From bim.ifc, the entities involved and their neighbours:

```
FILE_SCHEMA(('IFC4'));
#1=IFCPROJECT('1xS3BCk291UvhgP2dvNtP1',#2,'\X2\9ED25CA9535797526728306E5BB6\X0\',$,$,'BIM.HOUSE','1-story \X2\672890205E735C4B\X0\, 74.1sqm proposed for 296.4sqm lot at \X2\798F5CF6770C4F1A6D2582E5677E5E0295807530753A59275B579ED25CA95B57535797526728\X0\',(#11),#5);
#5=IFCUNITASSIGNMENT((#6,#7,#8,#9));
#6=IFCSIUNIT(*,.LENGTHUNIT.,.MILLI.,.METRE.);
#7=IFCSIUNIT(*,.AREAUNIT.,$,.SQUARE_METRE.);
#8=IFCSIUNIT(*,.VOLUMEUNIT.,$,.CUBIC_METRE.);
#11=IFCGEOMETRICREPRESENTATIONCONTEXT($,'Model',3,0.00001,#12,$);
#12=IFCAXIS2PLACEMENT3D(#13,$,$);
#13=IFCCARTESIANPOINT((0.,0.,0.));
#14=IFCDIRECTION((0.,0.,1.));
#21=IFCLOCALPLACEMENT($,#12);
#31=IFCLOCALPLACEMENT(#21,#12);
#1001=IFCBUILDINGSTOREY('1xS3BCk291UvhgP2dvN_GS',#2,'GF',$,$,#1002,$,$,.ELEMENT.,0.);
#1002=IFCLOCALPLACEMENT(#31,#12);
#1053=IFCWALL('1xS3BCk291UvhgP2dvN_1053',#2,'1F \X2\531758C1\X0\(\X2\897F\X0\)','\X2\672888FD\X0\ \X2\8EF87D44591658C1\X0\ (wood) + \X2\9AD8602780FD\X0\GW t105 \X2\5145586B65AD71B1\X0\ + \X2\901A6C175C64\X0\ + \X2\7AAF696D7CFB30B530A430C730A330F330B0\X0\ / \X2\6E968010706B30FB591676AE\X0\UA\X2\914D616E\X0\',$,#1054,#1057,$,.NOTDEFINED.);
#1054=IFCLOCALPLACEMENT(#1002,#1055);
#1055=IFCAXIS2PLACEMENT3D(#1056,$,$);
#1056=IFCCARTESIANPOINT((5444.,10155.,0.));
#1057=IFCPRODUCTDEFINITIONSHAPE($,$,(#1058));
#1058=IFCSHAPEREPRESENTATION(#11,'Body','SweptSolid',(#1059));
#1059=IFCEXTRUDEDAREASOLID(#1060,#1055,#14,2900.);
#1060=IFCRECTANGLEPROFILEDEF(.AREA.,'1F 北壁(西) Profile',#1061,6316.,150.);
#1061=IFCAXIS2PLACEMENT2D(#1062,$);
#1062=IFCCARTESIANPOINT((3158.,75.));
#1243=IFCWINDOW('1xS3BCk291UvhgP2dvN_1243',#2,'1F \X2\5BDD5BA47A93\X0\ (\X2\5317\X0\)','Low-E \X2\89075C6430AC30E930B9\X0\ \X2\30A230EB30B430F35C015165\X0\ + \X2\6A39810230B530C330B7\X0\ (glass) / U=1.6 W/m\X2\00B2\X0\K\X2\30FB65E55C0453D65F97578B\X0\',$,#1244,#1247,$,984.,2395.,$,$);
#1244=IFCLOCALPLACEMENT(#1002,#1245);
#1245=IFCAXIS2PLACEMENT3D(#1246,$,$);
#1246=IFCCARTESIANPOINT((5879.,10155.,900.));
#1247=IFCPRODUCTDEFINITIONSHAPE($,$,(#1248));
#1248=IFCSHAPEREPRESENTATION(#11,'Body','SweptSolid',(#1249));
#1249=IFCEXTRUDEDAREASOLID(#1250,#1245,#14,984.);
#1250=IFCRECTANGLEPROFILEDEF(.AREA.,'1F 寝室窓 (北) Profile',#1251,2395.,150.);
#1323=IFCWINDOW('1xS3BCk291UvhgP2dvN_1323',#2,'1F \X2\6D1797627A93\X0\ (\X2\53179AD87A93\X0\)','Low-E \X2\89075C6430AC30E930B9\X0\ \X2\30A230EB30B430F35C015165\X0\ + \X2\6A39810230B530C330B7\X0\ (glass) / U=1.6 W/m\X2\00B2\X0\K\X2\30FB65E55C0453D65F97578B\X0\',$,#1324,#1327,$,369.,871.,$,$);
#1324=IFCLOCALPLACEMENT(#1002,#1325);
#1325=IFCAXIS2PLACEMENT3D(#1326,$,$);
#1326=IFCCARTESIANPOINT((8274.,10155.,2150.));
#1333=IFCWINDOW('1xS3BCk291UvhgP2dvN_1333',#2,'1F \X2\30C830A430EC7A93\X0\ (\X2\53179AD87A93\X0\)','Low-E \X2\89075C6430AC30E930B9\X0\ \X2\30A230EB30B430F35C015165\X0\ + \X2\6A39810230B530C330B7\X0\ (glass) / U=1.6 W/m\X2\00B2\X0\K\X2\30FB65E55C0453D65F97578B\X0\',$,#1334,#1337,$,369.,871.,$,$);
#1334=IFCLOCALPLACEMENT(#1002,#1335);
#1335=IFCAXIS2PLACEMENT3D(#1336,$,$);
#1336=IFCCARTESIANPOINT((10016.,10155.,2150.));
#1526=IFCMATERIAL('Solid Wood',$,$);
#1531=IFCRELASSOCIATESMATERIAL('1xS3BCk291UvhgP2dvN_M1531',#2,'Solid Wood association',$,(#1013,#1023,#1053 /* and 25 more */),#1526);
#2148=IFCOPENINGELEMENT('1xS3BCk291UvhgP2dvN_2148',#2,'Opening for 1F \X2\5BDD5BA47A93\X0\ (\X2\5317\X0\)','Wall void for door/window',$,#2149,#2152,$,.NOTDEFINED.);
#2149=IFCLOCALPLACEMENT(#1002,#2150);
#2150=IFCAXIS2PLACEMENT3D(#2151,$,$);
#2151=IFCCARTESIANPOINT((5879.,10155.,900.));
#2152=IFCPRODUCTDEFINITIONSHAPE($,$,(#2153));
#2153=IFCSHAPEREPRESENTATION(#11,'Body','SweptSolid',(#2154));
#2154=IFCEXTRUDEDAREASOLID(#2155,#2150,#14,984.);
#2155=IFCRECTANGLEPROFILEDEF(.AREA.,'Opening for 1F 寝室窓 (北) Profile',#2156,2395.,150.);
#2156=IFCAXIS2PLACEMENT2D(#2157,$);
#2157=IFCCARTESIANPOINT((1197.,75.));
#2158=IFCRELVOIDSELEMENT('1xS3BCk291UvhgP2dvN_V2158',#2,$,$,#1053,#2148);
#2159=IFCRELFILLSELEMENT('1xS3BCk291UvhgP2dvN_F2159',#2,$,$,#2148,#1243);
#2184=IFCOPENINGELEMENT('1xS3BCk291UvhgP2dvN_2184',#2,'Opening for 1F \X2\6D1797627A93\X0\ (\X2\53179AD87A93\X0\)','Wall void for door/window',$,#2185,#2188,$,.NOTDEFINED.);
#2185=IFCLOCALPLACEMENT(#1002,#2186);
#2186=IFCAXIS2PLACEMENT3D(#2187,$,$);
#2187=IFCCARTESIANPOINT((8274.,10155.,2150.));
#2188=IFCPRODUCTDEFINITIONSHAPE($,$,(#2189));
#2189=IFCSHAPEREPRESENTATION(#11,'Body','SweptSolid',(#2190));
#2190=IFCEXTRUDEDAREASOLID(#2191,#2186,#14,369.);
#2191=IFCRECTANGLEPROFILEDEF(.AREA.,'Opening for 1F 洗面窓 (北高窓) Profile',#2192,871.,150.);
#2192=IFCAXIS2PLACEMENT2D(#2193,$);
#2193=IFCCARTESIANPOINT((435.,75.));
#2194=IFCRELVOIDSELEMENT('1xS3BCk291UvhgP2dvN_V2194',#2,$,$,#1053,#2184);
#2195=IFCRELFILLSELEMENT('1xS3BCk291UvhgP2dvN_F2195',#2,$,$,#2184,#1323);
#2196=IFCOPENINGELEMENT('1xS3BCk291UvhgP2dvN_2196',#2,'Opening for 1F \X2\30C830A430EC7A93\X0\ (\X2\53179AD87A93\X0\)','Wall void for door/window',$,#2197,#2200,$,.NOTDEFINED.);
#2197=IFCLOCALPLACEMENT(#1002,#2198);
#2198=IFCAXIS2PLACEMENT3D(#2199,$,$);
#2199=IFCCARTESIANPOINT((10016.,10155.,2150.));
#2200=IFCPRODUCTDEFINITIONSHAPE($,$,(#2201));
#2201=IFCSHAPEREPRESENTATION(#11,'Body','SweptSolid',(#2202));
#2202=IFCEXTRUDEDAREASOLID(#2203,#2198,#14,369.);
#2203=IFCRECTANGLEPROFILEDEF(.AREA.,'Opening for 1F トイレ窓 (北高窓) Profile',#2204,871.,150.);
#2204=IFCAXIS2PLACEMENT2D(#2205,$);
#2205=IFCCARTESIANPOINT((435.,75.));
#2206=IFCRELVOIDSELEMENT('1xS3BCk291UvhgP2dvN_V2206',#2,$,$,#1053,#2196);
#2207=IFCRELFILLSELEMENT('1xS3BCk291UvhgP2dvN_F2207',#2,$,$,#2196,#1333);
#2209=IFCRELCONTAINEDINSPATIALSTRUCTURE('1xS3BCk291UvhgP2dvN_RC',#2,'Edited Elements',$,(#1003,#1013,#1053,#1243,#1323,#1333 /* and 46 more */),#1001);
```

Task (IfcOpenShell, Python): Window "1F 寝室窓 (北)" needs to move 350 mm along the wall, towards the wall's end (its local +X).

```python
import ifcopenshell
import ifcopenshell.api.geometry
import ifcopenshell.util.placement
import ifcopenshell.util.unit

model = ifcopenshell.open("bim.ifc")
unit_scale = ifcopenshell.util.unit.calculate_unit_scale(model)

window = model.by_guid("1xS3BCk291UvhgP2dvN_1243")
opening = window.FillsVoids[0].RelatingOpeningElement
wall = opening.VoidsElements[0].RelatingBuildingElement

wall_matrix = ifcopenshell.util.placement.get_local_placement(wall.ObjectPlacement)
shift = wall_matrix[:3, 0] * 0.35 / unit_scale
before = ifcopenshell.util.placement.get_local_placement(window.ObjectPlacement)[:3, 3].copy()

# The window is not placed relative to its opening, so move both.
for product in (opening, window):
    matrix = ifcopenshell.util.placement.get_local_placement(product.ObjectPlacement)
    matrix[:3, 3] += shift
    ifcopenshell.api.geometry.edit_object_placement(model, product=product, matrix=matrix, is_si=False)

after = ifcopenshell.util.placement.get_local_placement(window.ObjectPlacement)[:3, 3]
print("window moved by", (after - before).round(3) + 0.0)

model.write("bim_updated.ifc")
```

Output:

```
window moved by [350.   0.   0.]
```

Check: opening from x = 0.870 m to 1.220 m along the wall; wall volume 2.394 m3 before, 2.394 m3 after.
